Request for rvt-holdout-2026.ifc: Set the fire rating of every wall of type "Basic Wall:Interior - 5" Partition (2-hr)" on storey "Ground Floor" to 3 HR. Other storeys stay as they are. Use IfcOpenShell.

First a look at what the model holds.

```python
import ifcopenshell
import ifcopenshell.util.element

model = ifcopenshell.open("rvt-holdout-2026.ifc")
print(model.schema)
storey = next(s for s in model.by_type("IfcBuildingStorey") if s.Name == "Ground Floor")
walls = [e for e in ifcopenshell.util.element.get_decomposition(storey) if e.is_a("IfcWall")]
seen = {}
for e in walls:
    element_type = ifcopenshell.util.element.get_type(e)
    key = (element_type.Name if element_type != e and element_type else None, ifcopenshell.util.element.get_pset(e, "Pset_WallCommon", "FireRating"))
    seen[key] = seen.get(key, 0) + 1
for (name, value), count in sorted(seen.items(), key=str):
    print(count, "x", name, "|", value)
```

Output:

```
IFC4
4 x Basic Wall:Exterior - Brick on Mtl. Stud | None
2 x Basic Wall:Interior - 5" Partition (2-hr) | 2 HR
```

```python
import ifcopenshell
import ifcopenshell.api.pset
import ifcopenshell.util.element

model = ifcopenshell.open("rvt-holdout-2026.ifc")

storey = next(s for s in model.by_type("IfcBuildingStorey") if s.Name == "Ground Floor")
walls = [e for e in ifcopenshell.util.element.get_decomposition(storey) if e.is_a("IfcWall")]

count = 0
for e in walls:
    element_type = ifcopenshell.util.element.get_type(e)
    if element_type in (None, e) or element_type.Name != 'Basic Wall:Interior - 5" Partition (2-hr)':
        continue
    # add_pset returns the element's existing set when there is one.
    pset = ifcopenshell.api.pset.add_pset(model, product=e, name="Pset_WallCommon")
    ifcopenshell.api.pset.edit_pset(model, pset=pset, properties={"FireRating": "3 HR"})
    count += 1

print(count, "walls updated")

model.write("rvt-holdout-2026_updated.ifc")
```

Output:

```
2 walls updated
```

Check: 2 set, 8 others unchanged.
